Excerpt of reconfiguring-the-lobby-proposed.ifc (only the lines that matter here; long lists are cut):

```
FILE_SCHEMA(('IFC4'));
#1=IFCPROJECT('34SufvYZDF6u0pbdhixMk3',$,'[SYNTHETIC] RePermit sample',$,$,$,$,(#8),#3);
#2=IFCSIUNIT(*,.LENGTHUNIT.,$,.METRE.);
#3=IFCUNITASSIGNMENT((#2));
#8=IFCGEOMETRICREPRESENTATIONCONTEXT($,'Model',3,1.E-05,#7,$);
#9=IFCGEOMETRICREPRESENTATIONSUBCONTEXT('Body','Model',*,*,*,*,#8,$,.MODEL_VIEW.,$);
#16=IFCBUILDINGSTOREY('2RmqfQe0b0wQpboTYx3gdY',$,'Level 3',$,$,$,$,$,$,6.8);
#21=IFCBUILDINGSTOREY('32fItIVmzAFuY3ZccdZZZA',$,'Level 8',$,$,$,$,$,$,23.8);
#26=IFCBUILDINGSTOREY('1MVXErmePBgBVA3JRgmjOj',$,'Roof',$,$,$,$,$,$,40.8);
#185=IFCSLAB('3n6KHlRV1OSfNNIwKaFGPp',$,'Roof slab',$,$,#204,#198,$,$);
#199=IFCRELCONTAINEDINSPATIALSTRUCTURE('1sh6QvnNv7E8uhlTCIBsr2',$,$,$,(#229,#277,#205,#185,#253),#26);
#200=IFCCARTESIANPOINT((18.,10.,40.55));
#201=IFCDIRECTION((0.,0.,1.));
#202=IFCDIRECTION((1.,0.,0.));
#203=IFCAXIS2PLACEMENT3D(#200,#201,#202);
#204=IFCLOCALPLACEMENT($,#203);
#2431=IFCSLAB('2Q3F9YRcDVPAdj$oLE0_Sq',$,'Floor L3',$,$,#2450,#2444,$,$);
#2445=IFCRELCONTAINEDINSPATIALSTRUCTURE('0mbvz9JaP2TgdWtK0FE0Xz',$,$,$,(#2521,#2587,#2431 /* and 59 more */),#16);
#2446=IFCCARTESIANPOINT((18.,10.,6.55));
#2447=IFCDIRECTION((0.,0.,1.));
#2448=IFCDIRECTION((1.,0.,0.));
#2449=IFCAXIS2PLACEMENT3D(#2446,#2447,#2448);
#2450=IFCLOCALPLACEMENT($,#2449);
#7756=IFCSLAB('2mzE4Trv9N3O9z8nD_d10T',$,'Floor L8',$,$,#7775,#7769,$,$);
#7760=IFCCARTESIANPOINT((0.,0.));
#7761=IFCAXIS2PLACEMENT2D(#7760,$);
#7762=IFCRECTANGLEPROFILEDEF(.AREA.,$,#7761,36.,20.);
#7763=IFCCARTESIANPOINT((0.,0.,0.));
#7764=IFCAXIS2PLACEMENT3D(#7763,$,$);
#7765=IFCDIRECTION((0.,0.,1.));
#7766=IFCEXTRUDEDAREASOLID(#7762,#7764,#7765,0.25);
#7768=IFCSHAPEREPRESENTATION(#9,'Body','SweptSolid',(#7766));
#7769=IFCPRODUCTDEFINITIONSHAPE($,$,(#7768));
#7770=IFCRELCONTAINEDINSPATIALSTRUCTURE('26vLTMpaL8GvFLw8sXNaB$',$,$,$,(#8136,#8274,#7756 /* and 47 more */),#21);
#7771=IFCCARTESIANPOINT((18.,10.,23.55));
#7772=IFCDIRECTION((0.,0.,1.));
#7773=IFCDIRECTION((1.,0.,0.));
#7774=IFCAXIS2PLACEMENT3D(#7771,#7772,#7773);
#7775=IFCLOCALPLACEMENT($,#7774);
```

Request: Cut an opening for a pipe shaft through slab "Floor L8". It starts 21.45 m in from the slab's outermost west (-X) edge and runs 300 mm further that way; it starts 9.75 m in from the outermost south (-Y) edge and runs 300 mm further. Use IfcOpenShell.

```python
import numpy as np
import ifcopenshell
import ifcopenshell.api.feature
import ifcopenshell.api.geometry
import ifcopenshell.api.root
import ifcopenshell.geom
import ifcopenshell.util.placement
import ifcopenshell.util.representation
import ifcopenshell.util.shape
import ifcopenshell.util.unit

model = ifcopenshell.open("reconfiguring-the-lobby-proposed.ifc")
unit_scale = ifcopenshell.util.unit.calculate_unit_scale(model)
settings = ifcopenshell.geom.settings()


def volume(element):
    """Net volume in cubic metres, openings subtracted."""
    shape = ifcopenshell.geom.create_shape(settings, element)
    return ifcopenshell.util.shape.get_volume(shape.geometry)


slab = model.by_id(7756)
before = volume(slab)

# Extent in the slab's own axes, in metres. The edges named are its -X and -Y sides.
slab_shape = ifcopenshell.geom.create_shape(settings, slab)
vertices = ifcopenshell.util.shape.get_vertices(slab_shape.geometry)
x_min, y_min, bottom = vertices.min(axis=0)
top = vertices[:, 2].max()

opening = ifcopenshell.api.root.create_entity(model, ifc_class="IfcOpeningElement", name="Pipe shaft opening", predefined_type="OPENING")
context = ifcopenshell.util.representation.get_context(model, "Model", "Body", "MODEL_VIEW")
width, depth = 0.3, 0.3
outline = [(0.0, 0.0), (width, 0.0), (width, depth), (0.0, depth), (0.0, 0.0)]
# Overshoot both faces by 50 mm so the cut is clean.
shape = ifcopenshell.api.geometry.add_slab_representation(
    model, context=context, depth=top - bottom + 0.1, polyline=outline
)
ifcopenshell.api.geometry.assign_representation(model, product=opening, representation=shape)

matrix = ifcopenshell.util.placement.get_local_placement(slab.ObjectPlacement)
matrix[:, 3] = matrix @ np.append(np.array([x_min + 21.45, y_min + 9.75, bottom - 0.05]) / unit_scale, 1.0)
ifcopenshell.api.geometry.edit_object_placement(model, product=opening, matrix=matrix, is_si=False)
ifcopenshell.api.feature.add_feature(model, feature=opening, element=slab)

after = volume(slab)

print(f"slab volume {before:.3f} -> {after:.3f} m3")

model.write("reconfiguring-the-lobby-proposed-out.ifc")
```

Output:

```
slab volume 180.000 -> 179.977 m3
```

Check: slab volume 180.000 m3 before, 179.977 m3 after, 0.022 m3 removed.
